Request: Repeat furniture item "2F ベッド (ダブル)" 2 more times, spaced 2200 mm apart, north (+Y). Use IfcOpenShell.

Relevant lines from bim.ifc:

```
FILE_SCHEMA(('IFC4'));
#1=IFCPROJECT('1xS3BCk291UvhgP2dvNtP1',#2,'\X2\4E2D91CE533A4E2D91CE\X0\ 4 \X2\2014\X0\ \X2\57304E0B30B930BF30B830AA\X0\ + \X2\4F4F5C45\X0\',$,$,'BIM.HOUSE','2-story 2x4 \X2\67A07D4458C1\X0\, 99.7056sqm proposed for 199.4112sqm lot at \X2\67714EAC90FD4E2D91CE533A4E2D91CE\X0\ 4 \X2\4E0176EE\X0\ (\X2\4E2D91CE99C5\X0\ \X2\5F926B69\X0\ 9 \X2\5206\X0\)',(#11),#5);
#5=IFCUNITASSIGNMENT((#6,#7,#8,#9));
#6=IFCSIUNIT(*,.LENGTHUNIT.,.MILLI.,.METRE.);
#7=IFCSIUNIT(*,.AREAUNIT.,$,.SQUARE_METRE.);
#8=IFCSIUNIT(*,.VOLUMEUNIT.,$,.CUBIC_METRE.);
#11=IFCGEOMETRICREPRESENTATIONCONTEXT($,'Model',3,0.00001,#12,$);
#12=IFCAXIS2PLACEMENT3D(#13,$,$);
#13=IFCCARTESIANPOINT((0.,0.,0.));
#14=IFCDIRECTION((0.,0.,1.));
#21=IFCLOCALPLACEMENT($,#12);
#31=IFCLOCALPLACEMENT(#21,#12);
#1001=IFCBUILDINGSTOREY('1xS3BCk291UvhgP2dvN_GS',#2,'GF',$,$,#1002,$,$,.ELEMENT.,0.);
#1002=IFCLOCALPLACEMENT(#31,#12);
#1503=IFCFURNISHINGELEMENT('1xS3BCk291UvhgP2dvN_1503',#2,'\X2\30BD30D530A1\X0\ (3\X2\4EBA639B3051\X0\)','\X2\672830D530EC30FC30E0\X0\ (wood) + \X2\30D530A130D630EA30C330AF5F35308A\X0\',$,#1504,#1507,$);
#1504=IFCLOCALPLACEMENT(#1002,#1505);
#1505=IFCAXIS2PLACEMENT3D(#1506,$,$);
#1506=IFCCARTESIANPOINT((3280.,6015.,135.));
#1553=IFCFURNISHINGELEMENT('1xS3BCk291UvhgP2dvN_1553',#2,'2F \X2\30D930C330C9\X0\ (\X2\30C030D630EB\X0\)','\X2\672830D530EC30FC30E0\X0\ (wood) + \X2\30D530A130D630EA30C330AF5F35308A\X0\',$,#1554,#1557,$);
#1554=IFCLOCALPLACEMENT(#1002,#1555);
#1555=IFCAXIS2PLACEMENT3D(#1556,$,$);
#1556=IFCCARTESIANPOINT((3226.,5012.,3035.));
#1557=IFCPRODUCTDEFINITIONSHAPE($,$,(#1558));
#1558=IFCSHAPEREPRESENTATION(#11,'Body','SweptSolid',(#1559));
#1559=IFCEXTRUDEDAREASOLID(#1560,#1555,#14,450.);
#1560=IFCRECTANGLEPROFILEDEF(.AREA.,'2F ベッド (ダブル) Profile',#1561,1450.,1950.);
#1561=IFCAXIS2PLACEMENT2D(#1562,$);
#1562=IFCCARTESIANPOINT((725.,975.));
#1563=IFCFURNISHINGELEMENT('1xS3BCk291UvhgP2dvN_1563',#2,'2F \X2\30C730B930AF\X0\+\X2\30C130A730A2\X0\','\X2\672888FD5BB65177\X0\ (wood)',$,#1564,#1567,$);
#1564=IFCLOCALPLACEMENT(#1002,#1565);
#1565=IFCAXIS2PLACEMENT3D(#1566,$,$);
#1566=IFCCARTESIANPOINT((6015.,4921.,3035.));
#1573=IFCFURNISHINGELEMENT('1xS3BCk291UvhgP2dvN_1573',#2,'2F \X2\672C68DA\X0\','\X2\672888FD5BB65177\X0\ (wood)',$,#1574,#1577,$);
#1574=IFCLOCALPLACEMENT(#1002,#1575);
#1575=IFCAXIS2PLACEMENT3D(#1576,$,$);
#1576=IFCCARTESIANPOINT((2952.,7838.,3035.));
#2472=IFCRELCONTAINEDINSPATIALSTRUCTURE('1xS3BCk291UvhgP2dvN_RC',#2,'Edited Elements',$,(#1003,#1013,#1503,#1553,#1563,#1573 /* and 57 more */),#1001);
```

```python
import numpy as np
import ifcopenshell
import ifcopenshell.api.geometry
import ifcopenshell.api.root
import ifcopenshell.util.element
import ifcopenshell.util.placement
import ifcopenshell.util.unit

model = ifcopenshell.open("bim.ifc")
unit_scale = ifcopenshell.util.unit.calculate_unit_scale(model)


def reuse_history(source, copy):
    """copy_class also copies each property set's owner history, people and application; keep the originals."""
    for rel in copy.IsDefinedBy:
        if rel.is_a("IfcRelDefinesByProperties") and (history := rel.RelatingPropertyDefinition.OwnerHistory):
            rel.RelatingPropertyDefinition.OwnerHistory = source.OwnerHistory
            ifcopenshell.util.element.remove_deep2(model, history)


source = model.by_guid("1xS3BCk291UvhgP2dvN_1553")
base = ifcopenshell.util.placement.get_local_placement(source.ObjectPlacement)
step = np.array([0.0, 1.0, 0.0]) * 2.2 / unit_scale

for i in range(1, 3):
    copy = ifcopenshell.api.root.copy_class(model, product=source)
    copy.Representation = ifcopenshell.util.element.copy_deep(
        model, source.Representation, exclude=["IfcGeometricRepresentationContext", "IfcRepresentationMap"]
    )
    reuse_history(source, copy)
    matrix = base.copy()
    matrix[:3, 3] += i * step
    print("added at", matrix[:3, 3].round(3) + 0.0)
    ifcopenshell.api.geometry.edit_object_placement(model, product=copy, matrix=matrix, is_si=False)

model.write("bim_updated.ifc")
```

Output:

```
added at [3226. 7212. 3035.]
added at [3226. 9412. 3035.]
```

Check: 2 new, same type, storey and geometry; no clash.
